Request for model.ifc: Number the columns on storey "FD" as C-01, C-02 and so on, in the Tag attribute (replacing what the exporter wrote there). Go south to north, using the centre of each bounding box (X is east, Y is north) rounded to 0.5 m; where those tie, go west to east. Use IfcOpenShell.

First a look at what the model holds.

```python
import ifcopenshell
import ifcopenshell.util.element
import ifcopenshell.util.placement

model = ifcopenshell.open("model.ifc")
print(model.schema)
storey = next(s for s in model.by_type("IfcBuildingStorey") if s.Name == "FD")
columns = [e for e in ifcopenshell.util.element.get_decomposition(storey) if e.is_a("IfcColumn")]
for e in sorted(columns, key=lambda e: e.id()):
    origin = ifcopenshell.util.placement.get_local_placement(e.ObjectPlacement)[:3, 3]
    print(e.id(), e.Tag, e.Name, origin.round(2) + 0.0, sep=" | ")
```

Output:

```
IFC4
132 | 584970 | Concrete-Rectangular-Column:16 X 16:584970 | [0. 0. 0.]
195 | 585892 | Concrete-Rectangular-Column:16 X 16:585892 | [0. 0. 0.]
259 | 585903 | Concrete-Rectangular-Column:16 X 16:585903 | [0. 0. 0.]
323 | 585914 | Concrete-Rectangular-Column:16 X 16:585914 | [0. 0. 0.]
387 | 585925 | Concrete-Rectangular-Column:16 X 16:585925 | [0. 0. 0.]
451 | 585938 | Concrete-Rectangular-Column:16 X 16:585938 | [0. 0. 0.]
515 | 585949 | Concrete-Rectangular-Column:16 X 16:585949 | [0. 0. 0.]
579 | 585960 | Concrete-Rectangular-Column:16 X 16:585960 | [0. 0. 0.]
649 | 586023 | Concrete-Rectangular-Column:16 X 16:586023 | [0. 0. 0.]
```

```python
import ifcopenshell
import ifcopenshell.geom
import ifcopenshell.util.element
import ifcopenshell.util.shape

model = ifcopenshell.open("model.ifc")
settings = ifcopenshell.geom.settings()
settings.set("use-world-coords", True)


def centre(element):
    shape = ifcopenshell.geom.create_shape(settings, element)
    return ifcopenshell.util.shape.get_bbox_centroid(shape.geometry)


storey = next(s for s in model.by_type("IfcBuildingStorey") if s.Name == "FD")
columns = [e for e in ifcopenshell.util.element.get_decomposition(storey) if e.is_a("IfcColumn")]

# Insertion points can sit at a corner or the storey origin, so sort by the geometry (in metres).
centres = {e: centre(e) for e in columns}
columns.sort(key=lambda e: (round(centres[e][1] / 0.5), centres[e][0]))

for i, e in enumerate(columns, start=1):
    number = f"C-{i:02d}"
    e.Tag = number
    print(e.id(), number)

model.write("model_rev.ifc")
```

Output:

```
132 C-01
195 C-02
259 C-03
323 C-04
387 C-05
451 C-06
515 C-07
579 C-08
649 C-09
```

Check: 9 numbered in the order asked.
